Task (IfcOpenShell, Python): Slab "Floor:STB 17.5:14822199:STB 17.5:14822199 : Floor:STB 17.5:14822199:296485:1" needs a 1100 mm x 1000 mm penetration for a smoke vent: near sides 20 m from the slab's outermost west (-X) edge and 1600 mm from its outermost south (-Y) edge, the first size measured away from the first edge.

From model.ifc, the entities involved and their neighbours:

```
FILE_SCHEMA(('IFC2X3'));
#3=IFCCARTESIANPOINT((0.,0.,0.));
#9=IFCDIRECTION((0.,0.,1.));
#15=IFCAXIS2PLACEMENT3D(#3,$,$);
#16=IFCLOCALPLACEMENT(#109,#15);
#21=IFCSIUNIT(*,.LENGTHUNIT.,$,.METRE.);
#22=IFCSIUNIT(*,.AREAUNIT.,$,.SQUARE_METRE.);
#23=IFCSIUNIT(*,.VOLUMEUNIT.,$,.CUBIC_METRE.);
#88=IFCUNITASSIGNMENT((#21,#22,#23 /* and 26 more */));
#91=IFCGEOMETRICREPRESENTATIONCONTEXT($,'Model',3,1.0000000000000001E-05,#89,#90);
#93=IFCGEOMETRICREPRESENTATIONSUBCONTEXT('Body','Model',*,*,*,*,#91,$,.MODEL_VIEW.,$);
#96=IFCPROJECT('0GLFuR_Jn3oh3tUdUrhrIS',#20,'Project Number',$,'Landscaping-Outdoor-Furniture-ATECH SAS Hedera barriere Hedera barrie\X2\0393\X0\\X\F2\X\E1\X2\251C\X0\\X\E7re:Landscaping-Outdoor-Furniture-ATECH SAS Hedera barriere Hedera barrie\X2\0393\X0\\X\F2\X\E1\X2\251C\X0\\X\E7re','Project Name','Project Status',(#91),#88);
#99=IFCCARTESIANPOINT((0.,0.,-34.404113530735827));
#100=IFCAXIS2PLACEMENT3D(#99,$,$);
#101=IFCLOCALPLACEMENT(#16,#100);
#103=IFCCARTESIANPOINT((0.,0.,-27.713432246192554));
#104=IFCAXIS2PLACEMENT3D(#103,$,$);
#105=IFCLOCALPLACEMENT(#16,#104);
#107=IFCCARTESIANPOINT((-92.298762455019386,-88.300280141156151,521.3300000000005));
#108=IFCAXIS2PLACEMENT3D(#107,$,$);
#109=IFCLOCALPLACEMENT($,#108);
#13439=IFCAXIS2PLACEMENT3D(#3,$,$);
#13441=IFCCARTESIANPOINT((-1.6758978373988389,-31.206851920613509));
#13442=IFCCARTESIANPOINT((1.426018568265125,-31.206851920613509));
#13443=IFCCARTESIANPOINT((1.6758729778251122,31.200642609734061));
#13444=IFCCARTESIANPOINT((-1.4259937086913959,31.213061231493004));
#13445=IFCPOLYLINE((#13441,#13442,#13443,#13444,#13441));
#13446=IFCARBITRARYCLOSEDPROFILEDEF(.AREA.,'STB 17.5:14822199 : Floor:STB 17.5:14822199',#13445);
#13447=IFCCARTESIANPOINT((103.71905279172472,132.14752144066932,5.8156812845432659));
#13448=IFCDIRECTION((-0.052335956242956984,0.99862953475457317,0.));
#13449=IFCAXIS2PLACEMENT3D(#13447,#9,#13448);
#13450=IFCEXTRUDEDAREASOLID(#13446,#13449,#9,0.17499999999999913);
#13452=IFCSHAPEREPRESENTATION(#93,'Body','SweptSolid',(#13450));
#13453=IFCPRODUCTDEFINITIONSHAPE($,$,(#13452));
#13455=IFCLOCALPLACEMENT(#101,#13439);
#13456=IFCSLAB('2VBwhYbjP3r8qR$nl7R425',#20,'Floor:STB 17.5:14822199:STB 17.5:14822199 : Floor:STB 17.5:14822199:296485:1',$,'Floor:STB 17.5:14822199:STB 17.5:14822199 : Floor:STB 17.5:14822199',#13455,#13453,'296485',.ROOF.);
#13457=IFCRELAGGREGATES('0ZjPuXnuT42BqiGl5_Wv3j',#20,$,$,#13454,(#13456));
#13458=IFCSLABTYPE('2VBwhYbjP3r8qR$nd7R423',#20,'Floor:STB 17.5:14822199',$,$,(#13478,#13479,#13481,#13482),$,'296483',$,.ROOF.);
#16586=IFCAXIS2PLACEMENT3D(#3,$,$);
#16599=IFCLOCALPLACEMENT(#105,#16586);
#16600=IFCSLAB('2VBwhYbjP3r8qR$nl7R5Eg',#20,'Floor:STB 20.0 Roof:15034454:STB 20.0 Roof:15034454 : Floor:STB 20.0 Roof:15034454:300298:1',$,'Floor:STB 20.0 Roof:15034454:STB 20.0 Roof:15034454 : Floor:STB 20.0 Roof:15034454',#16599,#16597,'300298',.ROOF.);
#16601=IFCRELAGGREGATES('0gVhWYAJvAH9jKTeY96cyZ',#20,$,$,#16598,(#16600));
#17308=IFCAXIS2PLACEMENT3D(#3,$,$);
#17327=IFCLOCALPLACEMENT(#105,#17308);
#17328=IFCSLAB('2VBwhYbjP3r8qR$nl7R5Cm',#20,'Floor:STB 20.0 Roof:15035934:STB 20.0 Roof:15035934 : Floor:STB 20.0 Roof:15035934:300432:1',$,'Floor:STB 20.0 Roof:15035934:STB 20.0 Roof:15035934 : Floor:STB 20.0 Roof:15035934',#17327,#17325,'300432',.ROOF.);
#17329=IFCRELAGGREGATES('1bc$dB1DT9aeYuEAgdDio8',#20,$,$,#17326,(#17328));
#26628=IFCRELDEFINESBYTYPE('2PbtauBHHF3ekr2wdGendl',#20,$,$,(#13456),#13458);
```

```python
import numpy as np
import ifcopenshell
import ifcopenshell.api.feature
import ifcopenshell.api.geometry
import ifcopenshell.api.root
import ifcopenshell.geom
import ifcopenshell.util.placement
import ifcopenshell.util.representation
import ifcopenshell.util.shape
import ifcopenshell.util.unit

model = ifcopenshell.open("model.ifc")
unit_scale = ifcopenshell.util.unit.calculate_unit_scale(model)
settings = ifcopenshell.geom.settings()


def volume(element):
    """Net volume in cubic metres, openings subtracted."""
    shape = ifcopenshell.geom.create_shape(settings, element)
    return ifcopenshell.util.shape.get_volume(shape.geometry)


slab = model.by_id(13456)
before = volume(slab)

# Extent in the slab's own axes, in metres. The edges named are its -X and -Y sides.
slab_shape = ifcopenshell.geom.create_shape(settings, slab)
vertices = ifcopenshell.util.shape.get_vertices(slab_shape.geometry)
x_min, y_min, bottom = vertices.min(axis=0)
top = vertices[:, 2].max()

opening = ifcopenshell.api.root.create_entity(model, ifc_class="IfcOpeningElement", name="Smoke vent opening")
context = ifcopenshell.util.representation.get_context(model, "Model", "Body", "MODEL_VIEW")
width, depth = 1.1, 1
outline = [(0.0, 0.0), (width, 0.0), (width, depth), (0.0, depth), (0.0, 0.0)]
# Overshoot both faces by 50 mm so the cut is clean.
shape = ifcopenshell.api.geometry.add_slab_representation(
    model, context=context, depth=top - bottom + 0.1, polyline=outline
)
ifcopenshell.api.geometry.assign_representation(model, product=opening, representation=shape)

matrix = ifcopenshell.util.placement.get_local_placement(slab.ObjectPlacement)
matrix[:, 3] = matrix @ np.append(np.array([x_min + 20, y_min + 1.6, bottom - 0.05]) / unit_scale, 1.0)
ifcopenshell.api.geometry.edit_object_placement(model, product=opening, matrix=matrix, is_si=False)
ifcopenshell.api.feature.add_feature(model, feature=opening, element=slab)

after = volume(slab)

print(f"slab volume {before:.3f} -> {after:.3f} m3")

model.write("model_edited.ifc")
```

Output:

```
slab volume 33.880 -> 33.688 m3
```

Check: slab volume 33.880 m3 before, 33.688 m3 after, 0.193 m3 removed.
